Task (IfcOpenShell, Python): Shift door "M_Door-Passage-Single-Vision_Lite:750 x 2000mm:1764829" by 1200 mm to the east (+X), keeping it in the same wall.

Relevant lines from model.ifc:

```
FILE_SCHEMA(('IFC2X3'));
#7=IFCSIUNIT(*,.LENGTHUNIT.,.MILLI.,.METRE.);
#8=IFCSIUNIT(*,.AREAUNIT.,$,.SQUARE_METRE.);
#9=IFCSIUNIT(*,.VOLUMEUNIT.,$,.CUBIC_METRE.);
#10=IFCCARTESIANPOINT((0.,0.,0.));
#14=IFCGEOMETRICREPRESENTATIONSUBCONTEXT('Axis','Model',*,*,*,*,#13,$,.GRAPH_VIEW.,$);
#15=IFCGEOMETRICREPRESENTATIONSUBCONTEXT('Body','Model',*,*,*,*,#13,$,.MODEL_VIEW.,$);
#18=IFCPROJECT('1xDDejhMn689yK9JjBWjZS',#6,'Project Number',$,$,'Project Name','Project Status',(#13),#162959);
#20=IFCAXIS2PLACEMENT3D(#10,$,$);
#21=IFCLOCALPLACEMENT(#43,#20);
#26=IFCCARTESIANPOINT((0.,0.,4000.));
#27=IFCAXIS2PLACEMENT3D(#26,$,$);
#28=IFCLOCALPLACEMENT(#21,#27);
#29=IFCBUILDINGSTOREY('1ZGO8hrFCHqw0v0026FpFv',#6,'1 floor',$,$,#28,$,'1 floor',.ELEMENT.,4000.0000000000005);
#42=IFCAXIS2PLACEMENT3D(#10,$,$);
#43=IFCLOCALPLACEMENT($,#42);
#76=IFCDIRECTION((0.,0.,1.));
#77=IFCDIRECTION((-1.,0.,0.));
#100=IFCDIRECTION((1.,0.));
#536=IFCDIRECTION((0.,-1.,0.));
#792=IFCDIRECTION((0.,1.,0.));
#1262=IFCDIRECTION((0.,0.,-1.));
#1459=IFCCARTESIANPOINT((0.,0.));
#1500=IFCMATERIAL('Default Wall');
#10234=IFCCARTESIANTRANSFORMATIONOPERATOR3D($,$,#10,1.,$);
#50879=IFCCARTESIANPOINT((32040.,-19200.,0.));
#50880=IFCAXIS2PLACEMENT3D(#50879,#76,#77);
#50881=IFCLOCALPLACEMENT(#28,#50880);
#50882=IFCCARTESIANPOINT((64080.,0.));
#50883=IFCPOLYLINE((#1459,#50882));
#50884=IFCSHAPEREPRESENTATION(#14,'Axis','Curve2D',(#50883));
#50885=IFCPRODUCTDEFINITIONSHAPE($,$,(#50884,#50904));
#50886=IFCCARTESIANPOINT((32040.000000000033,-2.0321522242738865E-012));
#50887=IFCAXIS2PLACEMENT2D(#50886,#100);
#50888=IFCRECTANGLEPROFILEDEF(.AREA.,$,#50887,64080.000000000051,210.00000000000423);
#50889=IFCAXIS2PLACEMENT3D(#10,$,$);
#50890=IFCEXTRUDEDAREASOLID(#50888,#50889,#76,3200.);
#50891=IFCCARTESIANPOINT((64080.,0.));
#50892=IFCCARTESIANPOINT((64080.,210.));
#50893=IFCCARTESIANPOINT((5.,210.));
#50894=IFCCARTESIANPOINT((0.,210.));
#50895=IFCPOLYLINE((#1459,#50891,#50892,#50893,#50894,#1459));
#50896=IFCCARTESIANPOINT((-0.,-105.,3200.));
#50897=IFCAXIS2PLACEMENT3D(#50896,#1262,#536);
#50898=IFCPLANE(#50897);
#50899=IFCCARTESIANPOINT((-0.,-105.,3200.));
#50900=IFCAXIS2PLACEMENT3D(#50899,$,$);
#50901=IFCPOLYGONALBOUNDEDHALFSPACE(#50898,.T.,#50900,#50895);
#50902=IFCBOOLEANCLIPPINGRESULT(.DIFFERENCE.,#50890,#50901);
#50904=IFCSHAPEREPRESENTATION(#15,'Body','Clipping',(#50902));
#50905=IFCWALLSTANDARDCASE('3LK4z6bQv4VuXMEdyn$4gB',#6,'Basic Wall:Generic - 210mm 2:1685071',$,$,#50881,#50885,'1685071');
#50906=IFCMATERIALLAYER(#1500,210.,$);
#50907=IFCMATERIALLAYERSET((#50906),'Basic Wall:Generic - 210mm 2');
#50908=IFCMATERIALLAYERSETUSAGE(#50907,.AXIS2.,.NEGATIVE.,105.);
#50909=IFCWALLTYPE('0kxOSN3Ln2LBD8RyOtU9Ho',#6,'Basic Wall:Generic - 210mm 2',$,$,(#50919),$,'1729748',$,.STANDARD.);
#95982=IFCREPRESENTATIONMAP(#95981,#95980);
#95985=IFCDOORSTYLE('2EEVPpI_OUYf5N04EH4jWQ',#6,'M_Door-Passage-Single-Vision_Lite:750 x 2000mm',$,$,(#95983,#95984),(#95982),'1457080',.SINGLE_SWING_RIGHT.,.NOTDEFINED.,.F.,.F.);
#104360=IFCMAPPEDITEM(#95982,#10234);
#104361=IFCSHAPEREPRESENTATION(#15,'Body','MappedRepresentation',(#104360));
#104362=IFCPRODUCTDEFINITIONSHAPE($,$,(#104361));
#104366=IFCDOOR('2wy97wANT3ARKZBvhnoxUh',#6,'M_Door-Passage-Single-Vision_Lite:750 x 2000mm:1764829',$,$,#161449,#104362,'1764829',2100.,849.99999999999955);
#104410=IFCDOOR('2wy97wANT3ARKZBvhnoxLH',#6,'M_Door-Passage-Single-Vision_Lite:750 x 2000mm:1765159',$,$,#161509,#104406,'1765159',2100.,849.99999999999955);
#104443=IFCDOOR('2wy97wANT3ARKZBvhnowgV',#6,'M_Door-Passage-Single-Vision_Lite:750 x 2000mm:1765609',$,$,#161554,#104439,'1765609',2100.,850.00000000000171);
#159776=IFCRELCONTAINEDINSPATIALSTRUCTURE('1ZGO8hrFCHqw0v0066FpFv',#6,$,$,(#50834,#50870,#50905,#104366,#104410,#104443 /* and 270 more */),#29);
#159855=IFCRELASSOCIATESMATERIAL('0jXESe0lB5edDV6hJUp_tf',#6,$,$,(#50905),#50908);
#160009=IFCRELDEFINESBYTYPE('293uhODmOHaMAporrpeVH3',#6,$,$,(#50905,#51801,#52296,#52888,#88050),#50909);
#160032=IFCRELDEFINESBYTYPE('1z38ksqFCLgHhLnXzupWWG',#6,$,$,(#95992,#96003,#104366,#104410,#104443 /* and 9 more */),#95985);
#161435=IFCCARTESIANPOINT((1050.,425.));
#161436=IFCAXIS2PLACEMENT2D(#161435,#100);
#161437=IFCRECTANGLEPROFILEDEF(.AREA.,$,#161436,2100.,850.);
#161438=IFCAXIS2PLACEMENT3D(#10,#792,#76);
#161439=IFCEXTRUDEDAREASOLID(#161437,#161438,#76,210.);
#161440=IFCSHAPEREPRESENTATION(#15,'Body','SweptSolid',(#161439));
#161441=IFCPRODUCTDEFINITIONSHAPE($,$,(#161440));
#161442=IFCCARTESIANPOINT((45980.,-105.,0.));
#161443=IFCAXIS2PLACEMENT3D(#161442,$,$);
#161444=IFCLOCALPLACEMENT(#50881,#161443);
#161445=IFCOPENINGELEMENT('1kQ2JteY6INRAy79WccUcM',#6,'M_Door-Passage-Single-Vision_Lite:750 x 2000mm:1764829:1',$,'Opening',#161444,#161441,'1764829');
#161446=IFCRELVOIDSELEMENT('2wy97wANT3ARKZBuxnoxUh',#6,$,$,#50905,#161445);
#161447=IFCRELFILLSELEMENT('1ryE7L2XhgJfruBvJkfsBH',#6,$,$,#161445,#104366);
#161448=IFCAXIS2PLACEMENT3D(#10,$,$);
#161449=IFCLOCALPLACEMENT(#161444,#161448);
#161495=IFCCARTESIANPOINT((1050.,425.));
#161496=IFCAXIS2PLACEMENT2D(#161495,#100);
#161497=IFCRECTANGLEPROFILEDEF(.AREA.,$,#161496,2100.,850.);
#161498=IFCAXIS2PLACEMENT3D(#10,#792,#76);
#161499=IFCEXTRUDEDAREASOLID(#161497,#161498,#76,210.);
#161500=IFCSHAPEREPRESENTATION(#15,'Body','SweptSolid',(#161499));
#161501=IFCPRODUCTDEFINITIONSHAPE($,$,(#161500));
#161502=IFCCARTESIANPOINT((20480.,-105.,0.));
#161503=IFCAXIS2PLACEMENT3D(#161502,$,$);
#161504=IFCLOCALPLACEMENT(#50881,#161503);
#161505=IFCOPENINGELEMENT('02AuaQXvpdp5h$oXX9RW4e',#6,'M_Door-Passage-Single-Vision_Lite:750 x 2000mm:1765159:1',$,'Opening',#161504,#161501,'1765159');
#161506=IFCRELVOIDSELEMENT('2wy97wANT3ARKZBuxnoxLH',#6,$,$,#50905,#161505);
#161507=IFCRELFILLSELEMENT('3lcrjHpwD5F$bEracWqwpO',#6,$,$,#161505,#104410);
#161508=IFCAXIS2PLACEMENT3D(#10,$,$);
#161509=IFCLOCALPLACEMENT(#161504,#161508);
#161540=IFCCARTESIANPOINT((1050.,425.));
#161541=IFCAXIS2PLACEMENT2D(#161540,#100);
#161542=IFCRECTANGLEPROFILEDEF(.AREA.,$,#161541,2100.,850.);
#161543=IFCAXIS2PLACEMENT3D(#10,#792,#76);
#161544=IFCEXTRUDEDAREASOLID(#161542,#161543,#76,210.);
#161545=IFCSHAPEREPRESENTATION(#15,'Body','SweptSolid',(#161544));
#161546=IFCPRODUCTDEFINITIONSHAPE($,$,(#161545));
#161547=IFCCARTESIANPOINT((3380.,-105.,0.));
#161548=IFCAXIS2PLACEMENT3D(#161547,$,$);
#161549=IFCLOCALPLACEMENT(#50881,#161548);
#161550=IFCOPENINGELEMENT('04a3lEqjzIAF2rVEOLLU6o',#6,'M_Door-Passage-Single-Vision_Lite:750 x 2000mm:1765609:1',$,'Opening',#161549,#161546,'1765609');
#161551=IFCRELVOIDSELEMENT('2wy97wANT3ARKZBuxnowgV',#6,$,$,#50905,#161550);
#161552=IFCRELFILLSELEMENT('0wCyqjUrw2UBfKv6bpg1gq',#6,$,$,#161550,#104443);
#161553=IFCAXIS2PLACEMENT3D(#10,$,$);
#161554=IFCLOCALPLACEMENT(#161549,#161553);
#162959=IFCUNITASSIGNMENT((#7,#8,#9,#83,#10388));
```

```python
import ifcopenshell
import ifcopenshell.api.geometry
import ifcopenshell.util.placement
import ifcopenshell.util.unit

model = ifcopenshell.open("model.ifc")
unit_scale = ifcopenshell.util.unit.calculate_unit_scale(model)

door = model.by_guid("2wy97wANT3ARKZBvhnoxUh")
opening = door.FillsVoids[0].RelatingOpeningElement
wall = opening.VoidsElements[0].RelatingBuildingElement

wall_matrix = ifcopenshell.util.placement.get_local_placement(wall.ObjectPlacement)
shift = wall_matrix[:3, 0] * -1.2 / unit_scale
before = ifcopenshell.util.placement.get_local_placement(door.ObjectPlacement)[:3, 3].copy()

# The door is placed relative to its opening, so it follows when the opening moves.
matrix = ifcopenshell.util.placement.get_local_placement(opening.ObjectPlacement)
matrix[:3, 3] += shift
ifcopenshell.api.geometry.edit_object_placement(
    model, product=opening, matrix=matrix, is_si=False, should_transform_children=True
)

after = ifcopenshell.util.placement.get_local_placement(door.ObjectPlacement)[:3, 3]
print("door moved by", (after - before).round(3) + 0.0)

model.write("model_updated.ifc")
```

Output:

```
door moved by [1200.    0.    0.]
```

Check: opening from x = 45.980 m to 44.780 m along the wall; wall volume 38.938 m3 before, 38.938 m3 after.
